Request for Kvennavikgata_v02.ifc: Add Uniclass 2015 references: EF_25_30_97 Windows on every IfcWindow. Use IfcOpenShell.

First a look at what the model holds.

```python
import ifcopenshell

model = ifcopenshell.open("Kvennavikgata_v02.ifc")
print(model.schema)
print("classifications:", [c.Name for c in model.by_type("IfcClassification")])
for ifc_class in ("IfcDoor", "IfcRoof", "IfcStair", "IfcWall", "IfcWindow"):
    print(ifc_class, len(model.by_type(ifc_class)))
```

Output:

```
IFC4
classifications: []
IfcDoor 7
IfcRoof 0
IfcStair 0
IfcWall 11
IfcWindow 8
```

```python
import ifcopenshell
import ifcopenshell.api.classification

model = ifcopenshell.open("Kvennavikgata_v02.ifc")

system = ifcopenshell.api.classification.add_classification(model, classification="Uniclass 2015")

codes = {
    "IfcWindow": ("EF_25_30_97", "Windows"),
}
for ifc_class, (code, name) in codes.items():
    products = model.by_type(ifc_class)
    ifcopenshell.api.classification.add_reference(
        model, products=products, classification=system, identification=code, name=name
    )
    print(code, len(products))

model.write("Kvennavikgata_v02_edited.ifc")
```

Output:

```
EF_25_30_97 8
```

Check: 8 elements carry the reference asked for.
